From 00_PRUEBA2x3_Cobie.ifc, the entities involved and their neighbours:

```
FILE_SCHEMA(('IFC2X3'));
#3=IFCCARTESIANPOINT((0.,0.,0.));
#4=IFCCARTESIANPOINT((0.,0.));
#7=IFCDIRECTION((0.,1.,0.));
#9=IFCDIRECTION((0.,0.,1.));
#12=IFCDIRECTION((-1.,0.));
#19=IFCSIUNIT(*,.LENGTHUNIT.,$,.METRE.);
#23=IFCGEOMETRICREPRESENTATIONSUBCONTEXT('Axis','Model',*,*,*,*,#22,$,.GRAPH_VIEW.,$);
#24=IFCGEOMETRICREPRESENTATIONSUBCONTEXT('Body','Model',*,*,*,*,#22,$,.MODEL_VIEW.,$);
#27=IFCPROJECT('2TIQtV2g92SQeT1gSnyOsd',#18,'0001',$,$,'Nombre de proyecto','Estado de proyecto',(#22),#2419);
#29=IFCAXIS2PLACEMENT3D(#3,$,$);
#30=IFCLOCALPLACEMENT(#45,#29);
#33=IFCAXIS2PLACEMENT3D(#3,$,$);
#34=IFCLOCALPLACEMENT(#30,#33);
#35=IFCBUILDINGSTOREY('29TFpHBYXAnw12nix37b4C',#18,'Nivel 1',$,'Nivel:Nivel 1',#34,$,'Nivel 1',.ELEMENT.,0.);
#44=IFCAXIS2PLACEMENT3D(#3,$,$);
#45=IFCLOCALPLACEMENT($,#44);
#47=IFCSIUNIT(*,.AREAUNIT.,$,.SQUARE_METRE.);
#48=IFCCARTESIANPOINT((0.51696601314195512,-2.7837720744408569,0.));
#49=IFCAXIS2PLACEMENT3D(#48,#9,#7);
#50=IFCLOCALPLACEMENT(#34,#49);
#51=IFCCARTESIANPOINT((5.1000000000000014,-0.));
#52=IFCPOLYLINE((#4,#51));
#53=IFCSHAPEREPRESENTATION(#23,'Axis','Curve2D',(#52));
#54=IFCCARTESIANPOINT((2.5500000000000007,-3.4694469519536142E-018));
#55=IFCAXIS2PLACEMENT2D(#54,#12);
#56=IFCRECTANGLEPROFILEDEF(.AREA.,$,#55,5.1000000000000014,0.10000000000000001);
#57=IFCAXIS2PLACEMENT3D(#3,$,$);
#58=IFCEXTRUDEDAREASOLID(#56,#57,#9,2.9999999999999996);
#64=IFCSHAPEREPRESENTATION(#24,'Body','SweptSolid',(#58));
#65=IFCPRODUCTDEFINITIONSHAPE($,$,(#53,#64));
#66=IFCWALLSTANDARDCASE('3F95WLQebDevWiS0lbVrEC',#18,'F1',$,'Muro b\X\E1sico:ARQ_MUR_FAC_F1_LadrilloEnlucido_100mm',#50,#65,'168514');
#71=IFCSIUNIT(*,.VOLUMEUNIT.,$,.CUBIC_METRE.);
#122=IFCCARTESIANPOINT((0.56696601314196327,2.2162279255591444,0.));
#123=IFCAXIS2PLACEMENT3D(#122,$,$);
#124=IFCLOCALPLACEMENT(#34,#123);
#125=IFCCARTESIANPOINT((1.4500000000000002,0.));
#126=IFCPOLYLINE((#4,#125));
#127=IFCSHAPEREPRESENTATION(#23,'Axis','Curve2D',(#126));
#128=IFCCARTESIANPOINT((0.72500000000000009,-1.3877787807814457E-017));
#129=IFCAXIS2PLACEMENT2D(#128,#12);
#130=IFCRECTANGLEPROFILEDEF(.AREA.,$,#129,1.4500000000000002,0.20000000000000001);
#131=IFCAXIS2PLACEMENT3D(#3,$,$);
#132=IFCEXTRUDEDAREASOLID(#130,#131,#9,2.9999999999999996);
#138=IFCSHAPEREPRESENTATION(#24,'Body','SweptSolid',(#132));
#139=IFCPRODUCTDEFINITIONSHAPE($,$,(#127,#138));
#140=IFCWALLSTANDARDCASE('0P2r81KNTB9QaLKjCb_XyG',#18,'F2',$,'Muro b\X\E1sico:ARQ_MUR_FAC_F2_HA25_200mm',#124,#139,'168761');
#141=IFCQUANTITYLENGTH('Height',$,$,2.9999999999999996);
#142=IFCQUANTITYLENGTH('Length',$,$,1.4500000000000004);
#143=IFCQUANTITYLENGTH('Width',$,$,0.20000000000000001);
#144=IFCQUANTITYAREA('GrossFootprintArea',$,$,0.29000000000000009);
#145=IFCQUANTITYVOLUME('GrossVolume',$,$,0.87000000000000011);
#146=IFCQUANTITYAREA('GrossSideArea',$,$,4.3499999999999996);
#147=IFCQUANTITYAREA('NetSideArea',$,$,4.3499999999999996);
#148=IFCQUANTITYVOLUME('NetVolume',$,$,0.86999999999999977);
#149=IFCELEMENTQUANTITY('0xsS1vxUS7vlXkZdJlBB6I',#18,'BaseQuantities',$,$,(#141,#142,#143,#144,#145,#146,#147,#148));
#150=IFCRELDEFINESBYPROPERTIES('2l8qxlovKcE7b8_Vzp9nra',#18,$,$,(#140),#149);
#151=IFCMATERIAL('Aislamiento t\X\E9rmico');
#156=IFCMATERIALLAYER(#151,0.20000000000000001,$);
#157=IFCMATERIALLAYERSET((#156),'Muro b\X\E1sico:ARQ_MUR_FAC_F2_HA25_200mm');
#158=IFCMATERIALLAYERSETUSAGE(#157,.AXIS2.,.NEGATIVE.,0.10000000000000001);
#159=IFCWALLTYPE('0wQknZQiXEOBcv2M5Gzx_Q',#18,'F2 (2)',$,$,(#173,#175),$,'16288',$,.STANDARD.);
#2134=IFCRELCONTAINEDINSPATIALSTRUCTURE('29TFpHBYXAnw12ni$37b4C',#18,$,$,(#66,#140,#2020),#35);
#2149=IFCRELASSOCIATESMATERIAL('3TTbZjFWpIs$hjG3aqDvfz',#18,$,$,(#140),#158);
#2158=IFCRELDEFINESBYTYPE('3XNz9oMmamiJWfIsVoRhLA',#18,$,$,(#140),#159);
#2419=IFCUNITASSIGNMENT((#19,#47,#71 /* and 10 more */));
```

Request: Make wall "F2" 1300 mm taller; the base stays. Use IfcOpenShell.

```python
import ifcopenshell
import ifcopenshell.api.pset
import ifcopenshell.geom
import ifcopenshell.util.element
import ifcopenshell.util.representation
import ifcopenshell.util.shape
import ifcopenshell.util.unit

model = ifcopenshell.open("00_PRUEBA2x3_Cobie.ifc")
unit_scale = ifcopenshell.util.unit.calculate_unit_scale(model)
area_scale = ifcopenshell.util.unit.calculate_unit_scale(model, "AREAUNIT")
volume_scale = ifcopenshell.util.unit.calculate_unit_scale(model, "VOLUMEUNIT")
settings = ifcopenshell.geom.settings()


def volume(element):
    """Net volume in cubic metres, openings subtracted."""
    shape = ifcopenshell.geom.create_shape(settings, element)
    return ifcopenshell.util.shape.get_volume(shape.geometry)


wall = model.by_id(140)
before = volume(wall)

body = ifcopenshell.util.representation.get_representation(wall, "Model", "Body")
solid = body.Items[0]
old_height = solid.Depth
solid.Depth += 1.3 / unit_scale
after = volume(wall)
thickness = 0.2  # wall thickness in metres

# Update the stored height, areas and volumes.
qto = model.by_id(ifcopenshell.util.element.get_pset(wall, "BaseQuantities", should_inherit=False)["id"])
ifcopenshell.api.pset.edit_qto(model, qto=qto, properties={
    "Height": solid.Depth,
    "GrossVolume": ifcopenshell.util.element.get_pset(wall, "BaseQuantities", "GrossVolume") * solid.Depth / old_height,
    "GrossSideArea": ifcopenshell.util.element.get_pset(wall, "BaseQuantities", "GrossSideArea") * solid.Depth / old_height,
    "NetSideArea": after / thickness / area_scale,
    "NetVolume": after / volume_scale,
})

print(f"height {old_height:g} -> {solid.Depth:g}, volume {before:.3f} -> {after:.3f} m3")

model.write("00_PRUEBA2x3_Cobie-out.ifc")
```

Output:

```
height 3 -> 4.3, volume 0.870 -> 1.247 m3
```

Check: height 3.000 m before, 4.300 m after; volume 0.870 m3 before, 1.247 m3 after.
